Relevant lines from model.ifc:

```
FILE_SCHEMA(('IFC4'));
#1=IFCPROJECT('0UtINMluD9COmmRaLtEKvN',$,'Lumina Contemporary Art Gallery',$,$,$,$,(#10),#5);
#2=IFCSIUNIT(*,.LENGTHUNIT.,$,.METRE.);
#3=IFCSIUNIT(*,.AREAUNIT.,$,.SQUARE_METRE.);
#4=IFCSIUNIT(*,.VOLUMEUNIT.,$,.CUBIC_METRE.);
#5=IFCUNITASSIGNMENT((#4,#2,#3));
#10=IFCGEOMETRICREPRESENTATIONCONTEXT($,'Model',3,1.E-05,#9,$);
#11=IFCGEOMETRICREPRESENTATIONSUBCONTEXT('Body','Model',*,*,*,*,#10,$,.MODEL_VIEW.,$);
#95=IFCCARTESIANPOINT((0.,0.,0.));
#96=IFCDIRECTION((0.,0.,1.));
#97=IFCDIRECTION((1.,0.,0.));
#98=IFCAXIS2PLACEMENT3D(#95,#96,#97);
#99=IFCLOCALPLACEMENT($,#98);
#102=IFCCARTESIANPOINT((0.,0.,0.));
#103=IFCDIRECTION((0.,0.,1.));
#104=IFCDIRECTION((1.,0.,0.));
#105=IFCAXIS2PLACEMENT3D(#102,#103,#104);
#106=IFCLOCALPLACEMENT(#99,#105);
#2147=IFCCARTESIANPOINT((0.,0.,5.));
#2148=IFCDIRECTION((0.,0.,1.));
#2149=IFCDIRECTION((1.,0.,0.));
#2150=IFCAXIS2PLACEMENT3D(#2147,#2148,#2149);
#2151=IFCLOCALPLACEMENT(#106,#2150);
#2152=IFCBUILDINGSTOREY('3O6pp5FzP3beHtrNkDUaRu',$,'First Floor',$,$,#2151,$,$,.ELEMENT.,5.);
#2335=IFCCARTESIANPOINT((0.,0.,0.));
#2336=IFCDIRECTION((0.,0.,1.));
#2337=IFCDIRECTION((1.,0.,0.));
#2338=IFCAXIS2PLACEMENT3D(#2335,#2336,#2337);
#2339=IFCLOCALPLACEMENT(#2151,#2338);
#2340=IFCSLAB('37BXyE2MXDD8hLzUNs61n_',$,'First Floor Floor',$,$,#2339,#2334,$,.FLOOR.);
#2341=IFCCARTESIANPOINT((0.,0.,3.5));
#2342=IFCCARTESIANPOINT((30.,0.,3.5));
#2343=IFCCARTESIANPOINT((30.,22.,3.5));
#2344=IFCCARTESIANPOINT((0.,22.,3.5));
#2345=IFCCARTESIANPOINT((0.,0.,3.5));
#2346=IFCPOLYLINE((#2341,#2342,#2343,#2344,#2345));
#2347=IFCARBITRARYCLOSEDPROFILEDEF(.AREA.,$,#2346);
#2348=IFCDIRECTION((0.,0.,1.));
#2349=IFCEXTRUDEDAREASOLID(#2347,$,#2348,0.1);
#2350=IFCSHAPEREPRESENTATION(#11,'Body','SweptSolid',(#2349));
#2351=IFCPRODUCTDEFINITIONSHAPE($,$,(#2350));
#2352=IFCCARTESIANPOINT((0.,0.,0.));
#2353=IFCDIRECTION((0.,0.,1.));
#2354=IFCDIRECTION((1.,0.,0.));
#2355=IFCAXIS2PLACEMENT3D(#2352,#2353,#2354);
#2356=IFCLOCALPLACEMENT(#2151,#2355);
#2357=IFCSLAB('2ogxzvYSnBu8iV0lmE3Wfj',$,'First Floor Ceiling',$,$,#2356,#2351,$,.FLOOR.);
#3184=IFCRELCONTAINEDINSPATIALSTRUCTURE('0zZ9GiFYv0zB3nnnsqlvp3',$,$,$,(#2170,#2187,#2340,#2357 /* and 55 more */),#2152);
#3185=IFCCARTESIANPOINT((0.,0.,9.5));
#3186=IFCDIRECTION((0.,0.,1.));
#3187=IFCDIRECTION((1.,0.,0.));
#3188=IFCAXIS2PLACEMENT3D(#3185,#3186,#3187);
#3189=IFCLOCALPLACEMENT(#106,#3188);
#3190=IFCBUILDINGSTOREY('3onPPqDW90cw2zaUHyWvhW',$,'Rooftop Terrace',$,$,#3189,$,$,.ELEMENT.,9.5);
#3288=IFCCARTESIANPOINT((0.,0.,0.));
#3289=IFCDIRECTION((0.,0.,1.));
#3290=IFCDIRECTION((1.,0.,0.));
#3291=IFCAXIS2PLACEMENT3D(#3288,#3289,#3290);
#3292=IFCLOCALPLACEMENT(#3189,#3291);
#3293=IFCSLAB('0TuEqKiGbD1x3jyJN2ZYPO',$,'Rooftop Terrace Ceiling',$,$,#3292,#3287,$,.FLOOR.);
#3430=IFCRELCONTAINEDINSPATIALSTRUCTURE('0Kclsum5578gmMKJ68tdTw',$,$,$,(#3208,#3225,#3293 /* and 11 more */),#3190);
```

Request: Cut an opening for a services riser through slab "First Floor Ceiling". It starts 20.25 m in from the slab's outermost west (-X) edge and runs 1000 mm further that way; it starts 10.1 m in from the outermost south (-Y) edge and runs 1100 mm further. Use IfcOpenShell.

```python
import numpy as np
import ifcopenshell
import ifcopenshell.api.feature
import ifcopenshell.api.geometry
import ifcopenshell.api.root
import ifcopenshell.geom
import ifcopenshell.util.placement
import ifcopenshell.util.representation
import ifcopenshell.util.shape
import ifcopenshell.util.unit

model = ifcopenshell.open("model.ifc")
unit_scale = ifcopenshell.util.unit.calculate_unit_scale(model)
settings = ifcopenshell.geom.settings()


def volume(element):
    """Net volume in cubic metres, openings subtracted."""
    shape = ifcopenshell.geom.create_shape(settings, element)
    return ifcopenshell.util.shape.get_volume(shape.geometry)


slab = model.by_guid("2ogxzvYSnBu8iV0lmE3Wfj")
before = volume(slab)

# Extent in the slab's own axes, in metres. The edges named are its -X and -Y sides.
slab_shape = ifcopenshell.geom.create_shape(settings, slab)
vertices = ifcopenshell.util.shape.get_vertices(slab_shape.geometry)
x_min, y_min, bottom = vertices.min(axis=0)
top = vertices[:, 2].max()

opening = ifcopenshell.api.root.create_entity(model, ifc_class="IfcOpeningElement", name="Services riser opening", predefined_type="OPENING")
context = ifcopenshell.util.representation.get_context(model, "Model", "Body", "MODEL_VIEW")
width, depth = 1, 1.1
outline = [(0.0, 0.0), (width, 0.0), (width, depth), (0.0, depth), (0.0, 0.0)]
# Overshoot both faces by 50 mm so the cut is clean.
shape = ifcopenshell.api.geometry.add_slab_representation(
    model, context=context, depth=top - bottom + 0.1, polyline=outline
)
ifcopenshell.api.geometry.assign_representation(model, product=opening, representation=shape)

matrix = ifcopenshell.util.placement.get_local_placement(slab.ObjectPlacement)
matrix[:, 3] = matrix @ np.append(np.array([x_min + 20.25, y_min + 10.1, bottom - 0.05]) / unit_scale, 1.0)
ifcopenshell.api.geometry.edit_object_placement(model, product=opening, matrix=matrix, is_si=False)
ifcopenshell.api.feature.add_feature(model, feature=opening, element=slab)

after = volume(slab)

print(f"slab volume {before:.3f} -> {after:.3f} m3")

model.write("model_v2.ifc")
```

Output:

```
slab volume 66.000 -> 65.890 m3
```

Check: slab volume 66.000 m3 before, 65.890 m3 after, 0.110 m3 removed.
